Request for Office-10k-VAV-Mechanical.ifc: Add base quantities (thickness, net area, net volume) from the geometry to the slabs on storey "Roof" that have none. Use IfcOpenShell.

First a look at what the model holds.

```python
import ifcopenshell
import ifcopenshell.util.element
import ifcopenshell.util.unit

model = ifcopenshell.open("Office-10k-VAV-Mechanical.ifc")
print(model.schema)
for unit_type in ("LENGTHUNIT", "AREAUNIT", "VOLUMEUNIT"):
    print(unit_type, ifcopenshell.util.unit.calculate_unit_scale(model, unit_type))
storey = next(s for s in model.by_type("IfcBuildingStorey") if s.Name == "Roof")
slabs = [e for e in ifcopenshell.util.element.get_decomposition(storey) if e.is_a("IfcSlab")]
for e in sorted(slabs, key=lambda e: e.id()):
    print(e.id(), e.is_a(), e.Name, list(ifcopenshell.util.element.get_psets(e, qtos_only=True)), sep=" | ")
```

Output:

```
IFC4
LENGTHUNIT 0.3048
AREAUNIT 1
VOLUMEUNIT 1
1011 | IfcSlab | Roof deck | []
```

```python
import ifcopenshell
import ifcopenshell.api.pset
import ifcopenshell.geom
import ifcopenshell.util.element
import ifcopenshell.util.shape
import ifcopenshell.util.unit

model = ifcopenshell.open("Office-10k-VAV-Mechanical.ifc")
unit_scale = ifcopenshell.util.unit.calculate_unit_scale(model)
area_scale = ifcopenshell.util.unit.calculate_unit_scale(model, "AREAUNIT")
volume_scale = ifcopenshell.util.unit.calculate_unit_scale(model, "VOLUMEUNIT")
settings = ifcopenshell.geom.settings()

storey = next(s for s in model.by_type("IfcBuildingStorey") if s.Name == "Roof")
slabs = [e for e in ifcopenshell.util.element.get_decomposition(storey) if e.is_a("IfcSlab")]

for e in sorted(slabs, key=lambda e: e.id()):
    if ifcopenshell.util.element.get_psets(e, qtos_only=True, should_inherit=False):
        continue
    # Geometry comes back in metres, in the element's own axes.
    shape = ifcopenshell.geom.create_shape(settings, e)
    values = {
        "Width": ifcopenshell.util.shape.get_z(shape.geometry) / unit_scale,
        "NetArea": ifcopenshell.util.shape.get_footprint_area(shape.geometry) / area_scale,
        "NetVolume": ifcopenshell.util.shape.get_volume(shape.geometry) / volume_scale,
    }
    qto = ifcopenshell.api.pset.add_qto(model, product=e, name="Qto_SlabBaseQuantities")
    ifcopenshell.api.pset.edit_qto(model, qto=qto, properties=values)
    print(e.id(), {k: round(v, 3) for k, v in values.items()})

model.write("Office-10k-VAV-Mechanical_edited.ifc")
```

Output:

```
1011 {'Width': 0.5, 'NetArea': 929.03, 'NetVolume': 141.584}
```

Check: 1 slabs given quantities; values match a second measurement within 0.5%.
